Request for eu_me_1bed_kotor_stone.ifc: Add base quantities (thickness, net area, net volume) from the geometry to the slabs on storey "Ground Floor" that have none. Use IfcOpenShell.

First a look at what the model holds.

```python
import ifcopenshell
import ifcopenshell.util.element
import ifcopenshell.util.unit

model = ifcopenshell.open("eu_me_1bed_kotor_stone.ifc")
print(model.schema)
for unit_type in ("LENGTHUNIT", "AREAUNIT", "VOLUMEUNIT"):
    print(unit_type, ifcopenshell.util.unit.calculate_unit_scale(model, unit_type))
storey = next(s for s in model.by_type("IfcBuildingStorey") if s.Name == "Ground Floor")
slabs = [e for e in ifcopenshell.util.element.get_decomposition(storey) if e.is_a("IfcSlab")]
for e in sorted(slabs, key=lambda e: e.id()):
    print(e.id(), e.is_a(), e.Name, list(ifcopenshell.util.element.get_psets(e, qtos_only=True)), sep=" | ")
```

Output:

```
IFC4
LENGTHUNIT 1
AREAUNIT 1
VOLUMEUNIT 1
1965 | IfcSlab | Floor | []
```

```python
import ifcopenshell
import ifcopenshell.api.pset
import ifcopenshell.geom
import ifcopenshell.util.element
import ifcopenshell.util.shape
import ifcopenshell.util.unit

model = ifcopenshell.open("eu_me_1bed_kotor_stone.ifc")
unit_scale = ifcopenshell.util.unit.calculate_unit_scale(model)
area_scale = ifcopenshell.util.unit.calculate_unit_scale(model, "AREAUNIT")
volume_scale = ifcopenshell.util.unit.calculate_unit_scale(model, "VOLUMEUNIT")
settings = ifcopenshell.geom.settings()

storey = next(s for s in model.by_type("IfcBuildingStorey") if s.Name == "Ground Floor")
slabs = [e for e in ifcopenshell.util.element.get_decomposition(storey) if e.is_a("IfcSlab")]

for e in sorted(slabs, key=lambda e: e.id()):
    if ifcopenshell.util.element.get_psets(e, qtos_only=True, should_inherit=False):
        continue
    # Geometry comes back in metres, in the element's own axes.
    shape = ifcopenshell.geom.create_shape(settings, e)
    values = {
        "Width": ifcopenshell.util.shape.get_z(shape.geometry) / unit_scale,
        "NetArea": ifcopenshell.util.shape.get_footprint_area(shape.geometry) / area_scale,
        "NetVolume": ifcopenshell.util.shape.get_volume(shape.geometry) / volume_scale,
    }
    qto = ifcopenshell.api.pset.add_qto(model, product=e, name="Qto_SlabBaseQuantities")
    ifcopenshell.api.pset.edit_qto(model, qto=qto, properties=values)
    print(e.id(), {k: round(v, 3) for k, v in values.items()})

model.write("eu_me_1bed_kotor_stone_updated.ifc")
```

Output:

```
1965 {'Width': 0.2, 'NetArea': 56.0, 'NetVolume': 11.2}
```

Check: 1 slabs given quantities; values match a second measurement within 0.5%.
